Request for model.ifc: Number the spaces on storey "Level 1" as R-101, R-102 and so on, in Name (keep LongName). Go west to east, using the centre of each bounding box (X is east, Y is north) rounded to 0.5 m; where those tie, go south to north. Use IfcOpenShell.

First a look at what the model holds.

```python
import ifcopenshell
import ifcopenshell.util.element
import ifcopenshell.util.placement

model = ifcopenshell.open("model.ifc")
print(model.schema)
storey = next(s for s in model.by_type("IfcBuildingStorey") if s.Name == "Level 1")
spaces = [e for e in ifcopenshell.util.element.get_decomposition(storey) if e.is_a("IfcSpace")]
for e in sorted(spaces, key=lambda e: e.id()):
    origin = ifcopenshell.util.placement.get_local_placement(e.ObjectPlacement)[:3, 3]
    print(e.id(), e.Name, e.LongName, origin.round(2) + 0.0, sep=" | ")
```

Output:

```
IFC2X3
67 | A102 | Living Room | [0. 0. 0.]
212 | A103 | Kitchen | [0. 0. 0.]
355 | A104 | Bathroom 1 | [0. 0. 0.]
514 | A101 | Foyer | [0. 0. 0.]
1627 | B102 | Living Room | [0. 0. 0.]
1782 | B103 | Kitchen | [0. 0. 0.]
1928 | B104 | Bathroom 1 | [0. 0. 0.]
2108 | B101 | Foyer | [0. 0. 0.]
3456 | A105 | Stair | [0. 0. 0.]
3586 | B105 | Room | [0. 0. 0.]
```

```python
import ifcopenshell
import ifcopenshell.geom
import ifcopenshell.util.element
import ifcopenshell.util.shape

model = ifcopenshell.open("model.ifc")
settings = ifcopenshell.geom.settings()
settings.set("use-world-coords", True)


def centre(element):
    shape = ifcopenshell.geom.create_shape(settings, element)
    return ifcopenshell.util.shape.get_bbox_centroid(shape.geometry)


storey = next(s for s in model.by_type("IfcBuildingStorey") if s.Name == "Level 1")
spaces = [e for e in ifcopenshell.util.element.get_decomposition(storey) if e.is_a("IfcSpace")]

# Insertion points can sit at a corner or the storey origin, so sort by the geometry (in metres).
centres = {e: centre(e) for e in spaces}
spaces.sort(key=lambda e: (round(centres[e][0] / 0.5), centres[e][1]))

for i, e in enumerate(spaces, start=1):
    number = f"R-1{i:02d}"
    e.Name = number
    print(e.id(), number)

model.write("model_v2.ifc")
```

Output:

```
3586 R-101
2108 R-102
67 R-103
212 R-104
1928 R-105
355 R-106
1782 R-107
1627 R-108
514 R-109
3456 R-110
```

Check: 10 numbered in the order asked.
